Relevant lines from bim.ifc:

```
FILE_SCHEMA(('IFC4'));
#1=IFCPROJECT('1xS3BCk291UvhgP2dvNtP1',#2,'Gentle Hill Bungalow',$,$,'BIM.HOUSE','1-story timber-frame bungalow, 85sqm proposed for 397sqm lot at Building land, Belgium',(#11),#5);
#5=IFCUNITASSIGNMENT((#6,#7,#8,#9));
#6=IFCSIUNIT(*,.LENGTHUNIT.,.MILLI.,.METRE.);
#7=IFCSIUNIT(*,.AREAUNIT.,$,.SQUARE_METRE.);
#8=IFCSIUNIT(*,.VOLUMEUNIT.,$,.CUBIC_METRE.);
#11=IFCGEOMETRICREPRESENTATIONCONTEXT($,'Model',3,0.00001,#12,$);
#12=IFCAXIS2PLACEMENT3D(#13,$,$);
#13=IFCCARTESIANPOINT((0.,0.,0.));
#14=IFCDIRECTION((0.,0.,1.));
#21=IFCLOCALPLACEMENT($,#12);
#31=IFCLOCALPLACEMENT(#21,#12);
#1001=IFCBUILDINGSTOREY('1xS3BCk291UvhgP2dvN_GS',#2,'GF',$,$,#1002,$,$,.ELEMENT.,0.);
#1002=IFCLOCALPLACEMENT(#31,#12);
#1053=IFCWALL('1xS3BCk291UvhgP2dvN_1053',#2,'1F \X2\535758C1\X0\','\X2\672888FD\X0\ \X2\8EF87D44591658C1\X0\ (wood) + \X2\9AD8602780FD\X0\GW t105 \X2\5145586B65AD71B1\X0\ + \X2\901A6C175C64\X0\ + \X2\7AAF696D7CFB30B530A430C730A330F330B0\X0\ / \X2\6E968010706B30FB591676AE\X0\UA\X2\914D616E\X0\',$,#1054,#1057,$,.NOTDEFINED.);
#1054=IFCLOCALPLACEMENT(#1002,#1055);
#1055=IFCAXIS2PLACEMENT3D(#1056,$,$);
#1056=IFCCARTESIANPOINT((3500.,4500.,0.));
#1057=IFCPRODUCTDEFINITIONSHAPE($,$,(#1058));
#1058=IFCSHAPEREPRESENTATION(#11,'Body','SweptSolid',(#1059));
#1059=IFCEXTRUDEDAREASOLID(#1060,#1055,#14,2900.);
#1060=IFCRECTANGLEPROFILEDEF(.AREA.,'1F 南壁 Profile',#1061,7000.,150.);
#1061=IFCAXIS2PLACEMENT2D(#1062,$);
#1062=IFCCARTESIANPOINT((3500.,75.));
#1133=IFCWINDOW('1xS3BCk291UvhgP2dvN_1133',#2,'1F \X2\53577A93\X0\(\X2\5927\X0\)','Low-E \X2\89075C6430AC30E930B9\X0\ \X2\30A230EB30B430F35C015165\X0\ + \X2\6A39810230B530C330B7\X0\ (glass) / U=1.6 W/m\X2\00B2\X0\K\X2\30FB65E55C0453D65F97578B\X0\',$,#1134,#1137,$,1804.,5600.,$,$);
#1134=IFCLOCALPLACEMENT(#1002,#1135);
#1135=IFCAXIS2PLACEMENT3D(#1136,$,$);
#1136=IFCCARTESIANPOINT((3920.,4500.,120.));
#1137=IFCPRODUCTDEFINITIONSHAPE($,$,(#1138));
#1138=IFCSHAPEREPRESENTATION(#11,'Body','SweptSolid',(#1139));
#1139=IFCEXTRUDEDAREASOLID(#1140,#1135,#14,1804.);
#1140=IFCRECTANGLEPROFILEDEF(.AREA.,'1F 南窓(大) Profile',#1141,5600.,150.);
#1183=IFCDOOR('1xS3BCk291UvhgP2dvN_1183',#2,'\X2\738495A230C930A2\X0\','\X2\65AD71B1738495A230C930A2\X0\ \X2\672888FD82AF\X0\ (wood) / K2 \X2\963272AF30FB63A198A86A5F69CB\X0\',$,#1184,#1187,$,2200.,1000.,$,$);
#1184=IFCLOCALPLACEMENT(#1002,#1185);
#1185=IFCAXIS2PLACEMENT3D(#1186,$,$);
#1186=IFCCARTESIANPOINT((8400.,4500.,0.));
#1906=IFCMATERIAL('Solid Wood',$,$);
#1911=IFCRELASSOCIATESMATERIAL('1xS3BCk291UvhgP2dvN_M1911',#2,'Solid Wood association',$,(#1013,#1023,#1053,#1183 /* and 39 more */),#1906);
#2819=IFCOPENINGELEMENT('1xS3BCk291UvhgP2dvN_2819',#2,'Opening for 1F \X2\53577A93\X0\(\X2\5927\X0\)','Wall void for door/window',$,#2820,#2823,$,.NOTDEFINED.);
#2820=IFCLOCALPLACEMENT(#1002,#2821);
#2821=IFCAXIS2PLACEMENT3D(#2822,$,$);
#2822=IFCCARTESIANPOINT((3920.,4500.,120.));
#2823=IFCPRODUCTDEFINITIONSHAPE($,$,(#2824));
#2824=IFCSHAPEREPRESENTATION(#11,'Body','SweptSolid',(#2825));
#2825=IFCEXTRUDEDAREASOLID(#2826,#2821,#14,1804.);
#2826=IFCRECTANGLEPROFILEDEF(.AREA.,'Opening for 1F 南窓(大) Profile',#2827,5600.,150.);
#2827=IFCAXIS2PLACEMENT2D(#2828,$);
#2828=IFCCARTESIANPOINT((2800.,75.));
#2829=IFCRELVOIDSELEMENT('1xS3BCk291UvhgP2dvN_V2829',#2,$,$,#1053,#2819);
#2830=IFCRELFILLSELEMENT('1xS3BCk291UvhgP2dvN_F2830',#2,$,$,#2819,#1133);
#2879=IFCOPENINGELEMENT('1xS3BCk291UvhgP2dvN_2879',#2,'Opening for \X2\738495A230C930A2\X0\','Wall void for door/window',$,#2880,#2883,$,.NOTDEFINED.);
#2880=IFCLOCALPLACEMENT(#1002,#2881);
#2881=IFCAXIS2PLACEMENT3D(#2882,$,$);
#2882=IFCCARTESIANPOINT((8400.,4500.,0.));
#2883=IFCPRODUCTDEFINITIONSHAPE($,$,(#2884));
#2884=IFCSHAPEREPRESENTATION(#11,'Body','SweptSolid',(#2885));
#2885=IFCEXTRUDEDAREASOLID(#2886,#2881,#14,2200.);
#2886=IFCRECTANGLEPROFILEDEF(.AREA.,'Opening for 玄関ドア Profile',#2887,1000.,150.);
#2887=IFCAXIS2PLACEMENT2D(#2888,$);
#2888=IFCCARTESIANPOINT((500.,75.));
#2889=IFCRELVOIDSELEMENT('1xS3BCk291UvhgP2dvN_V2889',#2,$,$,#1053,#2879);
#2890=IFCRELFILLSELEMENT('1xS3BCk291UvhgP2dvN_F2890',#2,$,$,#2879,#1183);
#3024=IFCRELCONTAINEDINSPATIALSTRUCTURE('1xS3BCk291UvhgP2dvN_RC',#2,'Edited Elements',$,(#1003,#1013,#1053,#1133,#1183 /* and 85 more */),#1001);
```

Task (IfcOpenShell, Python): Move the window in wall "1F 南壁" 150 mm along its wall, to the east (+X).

```python
import ifcopenshell
import ifcopenshell.api.geometry
import ifcopenshell.util.placement

model = ifcopenshell.open("bim.ifc")

window = model.by_guid("1xS3BCk291UvhgP2dvN_1133")
opening = window.FillsVoids[0].RelatingOpeningElement
wall = opening.VoidsElements[0].RelatingBuildingElement

wall_matrix = ifcopenshell.util.placement.get_local_placement(wall.ObjectPlacement)
shift = wall_matrix[:3, 0] * 150.0
before = ifcopenshell.util.placement.get_local_placement(window.ObjectPlacement)[:3, 3].copy()

# The window is not placed relative to its opening, so move both.
for product in (opening, window):
    matrix = ifcopenshell.util.placement.get_local_placement(product.ObjectPlacement)
    matrix[:3, 3] += shift
    ifcopenshell.api.geometry.edit_object_placement(model, product=product, matrix=matrix, is_si=False)

after = ifcopenshell.util.placement.get_local_placement(window.ObjectPlacement)[:3, 3]
print("window moved by", (after - before).round(3) + 0.0)

model.write("bim_v2.ifc")
```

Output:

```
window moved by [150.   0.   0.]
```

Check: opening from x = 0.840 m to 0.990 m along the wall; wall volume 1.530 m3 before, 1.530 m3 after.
